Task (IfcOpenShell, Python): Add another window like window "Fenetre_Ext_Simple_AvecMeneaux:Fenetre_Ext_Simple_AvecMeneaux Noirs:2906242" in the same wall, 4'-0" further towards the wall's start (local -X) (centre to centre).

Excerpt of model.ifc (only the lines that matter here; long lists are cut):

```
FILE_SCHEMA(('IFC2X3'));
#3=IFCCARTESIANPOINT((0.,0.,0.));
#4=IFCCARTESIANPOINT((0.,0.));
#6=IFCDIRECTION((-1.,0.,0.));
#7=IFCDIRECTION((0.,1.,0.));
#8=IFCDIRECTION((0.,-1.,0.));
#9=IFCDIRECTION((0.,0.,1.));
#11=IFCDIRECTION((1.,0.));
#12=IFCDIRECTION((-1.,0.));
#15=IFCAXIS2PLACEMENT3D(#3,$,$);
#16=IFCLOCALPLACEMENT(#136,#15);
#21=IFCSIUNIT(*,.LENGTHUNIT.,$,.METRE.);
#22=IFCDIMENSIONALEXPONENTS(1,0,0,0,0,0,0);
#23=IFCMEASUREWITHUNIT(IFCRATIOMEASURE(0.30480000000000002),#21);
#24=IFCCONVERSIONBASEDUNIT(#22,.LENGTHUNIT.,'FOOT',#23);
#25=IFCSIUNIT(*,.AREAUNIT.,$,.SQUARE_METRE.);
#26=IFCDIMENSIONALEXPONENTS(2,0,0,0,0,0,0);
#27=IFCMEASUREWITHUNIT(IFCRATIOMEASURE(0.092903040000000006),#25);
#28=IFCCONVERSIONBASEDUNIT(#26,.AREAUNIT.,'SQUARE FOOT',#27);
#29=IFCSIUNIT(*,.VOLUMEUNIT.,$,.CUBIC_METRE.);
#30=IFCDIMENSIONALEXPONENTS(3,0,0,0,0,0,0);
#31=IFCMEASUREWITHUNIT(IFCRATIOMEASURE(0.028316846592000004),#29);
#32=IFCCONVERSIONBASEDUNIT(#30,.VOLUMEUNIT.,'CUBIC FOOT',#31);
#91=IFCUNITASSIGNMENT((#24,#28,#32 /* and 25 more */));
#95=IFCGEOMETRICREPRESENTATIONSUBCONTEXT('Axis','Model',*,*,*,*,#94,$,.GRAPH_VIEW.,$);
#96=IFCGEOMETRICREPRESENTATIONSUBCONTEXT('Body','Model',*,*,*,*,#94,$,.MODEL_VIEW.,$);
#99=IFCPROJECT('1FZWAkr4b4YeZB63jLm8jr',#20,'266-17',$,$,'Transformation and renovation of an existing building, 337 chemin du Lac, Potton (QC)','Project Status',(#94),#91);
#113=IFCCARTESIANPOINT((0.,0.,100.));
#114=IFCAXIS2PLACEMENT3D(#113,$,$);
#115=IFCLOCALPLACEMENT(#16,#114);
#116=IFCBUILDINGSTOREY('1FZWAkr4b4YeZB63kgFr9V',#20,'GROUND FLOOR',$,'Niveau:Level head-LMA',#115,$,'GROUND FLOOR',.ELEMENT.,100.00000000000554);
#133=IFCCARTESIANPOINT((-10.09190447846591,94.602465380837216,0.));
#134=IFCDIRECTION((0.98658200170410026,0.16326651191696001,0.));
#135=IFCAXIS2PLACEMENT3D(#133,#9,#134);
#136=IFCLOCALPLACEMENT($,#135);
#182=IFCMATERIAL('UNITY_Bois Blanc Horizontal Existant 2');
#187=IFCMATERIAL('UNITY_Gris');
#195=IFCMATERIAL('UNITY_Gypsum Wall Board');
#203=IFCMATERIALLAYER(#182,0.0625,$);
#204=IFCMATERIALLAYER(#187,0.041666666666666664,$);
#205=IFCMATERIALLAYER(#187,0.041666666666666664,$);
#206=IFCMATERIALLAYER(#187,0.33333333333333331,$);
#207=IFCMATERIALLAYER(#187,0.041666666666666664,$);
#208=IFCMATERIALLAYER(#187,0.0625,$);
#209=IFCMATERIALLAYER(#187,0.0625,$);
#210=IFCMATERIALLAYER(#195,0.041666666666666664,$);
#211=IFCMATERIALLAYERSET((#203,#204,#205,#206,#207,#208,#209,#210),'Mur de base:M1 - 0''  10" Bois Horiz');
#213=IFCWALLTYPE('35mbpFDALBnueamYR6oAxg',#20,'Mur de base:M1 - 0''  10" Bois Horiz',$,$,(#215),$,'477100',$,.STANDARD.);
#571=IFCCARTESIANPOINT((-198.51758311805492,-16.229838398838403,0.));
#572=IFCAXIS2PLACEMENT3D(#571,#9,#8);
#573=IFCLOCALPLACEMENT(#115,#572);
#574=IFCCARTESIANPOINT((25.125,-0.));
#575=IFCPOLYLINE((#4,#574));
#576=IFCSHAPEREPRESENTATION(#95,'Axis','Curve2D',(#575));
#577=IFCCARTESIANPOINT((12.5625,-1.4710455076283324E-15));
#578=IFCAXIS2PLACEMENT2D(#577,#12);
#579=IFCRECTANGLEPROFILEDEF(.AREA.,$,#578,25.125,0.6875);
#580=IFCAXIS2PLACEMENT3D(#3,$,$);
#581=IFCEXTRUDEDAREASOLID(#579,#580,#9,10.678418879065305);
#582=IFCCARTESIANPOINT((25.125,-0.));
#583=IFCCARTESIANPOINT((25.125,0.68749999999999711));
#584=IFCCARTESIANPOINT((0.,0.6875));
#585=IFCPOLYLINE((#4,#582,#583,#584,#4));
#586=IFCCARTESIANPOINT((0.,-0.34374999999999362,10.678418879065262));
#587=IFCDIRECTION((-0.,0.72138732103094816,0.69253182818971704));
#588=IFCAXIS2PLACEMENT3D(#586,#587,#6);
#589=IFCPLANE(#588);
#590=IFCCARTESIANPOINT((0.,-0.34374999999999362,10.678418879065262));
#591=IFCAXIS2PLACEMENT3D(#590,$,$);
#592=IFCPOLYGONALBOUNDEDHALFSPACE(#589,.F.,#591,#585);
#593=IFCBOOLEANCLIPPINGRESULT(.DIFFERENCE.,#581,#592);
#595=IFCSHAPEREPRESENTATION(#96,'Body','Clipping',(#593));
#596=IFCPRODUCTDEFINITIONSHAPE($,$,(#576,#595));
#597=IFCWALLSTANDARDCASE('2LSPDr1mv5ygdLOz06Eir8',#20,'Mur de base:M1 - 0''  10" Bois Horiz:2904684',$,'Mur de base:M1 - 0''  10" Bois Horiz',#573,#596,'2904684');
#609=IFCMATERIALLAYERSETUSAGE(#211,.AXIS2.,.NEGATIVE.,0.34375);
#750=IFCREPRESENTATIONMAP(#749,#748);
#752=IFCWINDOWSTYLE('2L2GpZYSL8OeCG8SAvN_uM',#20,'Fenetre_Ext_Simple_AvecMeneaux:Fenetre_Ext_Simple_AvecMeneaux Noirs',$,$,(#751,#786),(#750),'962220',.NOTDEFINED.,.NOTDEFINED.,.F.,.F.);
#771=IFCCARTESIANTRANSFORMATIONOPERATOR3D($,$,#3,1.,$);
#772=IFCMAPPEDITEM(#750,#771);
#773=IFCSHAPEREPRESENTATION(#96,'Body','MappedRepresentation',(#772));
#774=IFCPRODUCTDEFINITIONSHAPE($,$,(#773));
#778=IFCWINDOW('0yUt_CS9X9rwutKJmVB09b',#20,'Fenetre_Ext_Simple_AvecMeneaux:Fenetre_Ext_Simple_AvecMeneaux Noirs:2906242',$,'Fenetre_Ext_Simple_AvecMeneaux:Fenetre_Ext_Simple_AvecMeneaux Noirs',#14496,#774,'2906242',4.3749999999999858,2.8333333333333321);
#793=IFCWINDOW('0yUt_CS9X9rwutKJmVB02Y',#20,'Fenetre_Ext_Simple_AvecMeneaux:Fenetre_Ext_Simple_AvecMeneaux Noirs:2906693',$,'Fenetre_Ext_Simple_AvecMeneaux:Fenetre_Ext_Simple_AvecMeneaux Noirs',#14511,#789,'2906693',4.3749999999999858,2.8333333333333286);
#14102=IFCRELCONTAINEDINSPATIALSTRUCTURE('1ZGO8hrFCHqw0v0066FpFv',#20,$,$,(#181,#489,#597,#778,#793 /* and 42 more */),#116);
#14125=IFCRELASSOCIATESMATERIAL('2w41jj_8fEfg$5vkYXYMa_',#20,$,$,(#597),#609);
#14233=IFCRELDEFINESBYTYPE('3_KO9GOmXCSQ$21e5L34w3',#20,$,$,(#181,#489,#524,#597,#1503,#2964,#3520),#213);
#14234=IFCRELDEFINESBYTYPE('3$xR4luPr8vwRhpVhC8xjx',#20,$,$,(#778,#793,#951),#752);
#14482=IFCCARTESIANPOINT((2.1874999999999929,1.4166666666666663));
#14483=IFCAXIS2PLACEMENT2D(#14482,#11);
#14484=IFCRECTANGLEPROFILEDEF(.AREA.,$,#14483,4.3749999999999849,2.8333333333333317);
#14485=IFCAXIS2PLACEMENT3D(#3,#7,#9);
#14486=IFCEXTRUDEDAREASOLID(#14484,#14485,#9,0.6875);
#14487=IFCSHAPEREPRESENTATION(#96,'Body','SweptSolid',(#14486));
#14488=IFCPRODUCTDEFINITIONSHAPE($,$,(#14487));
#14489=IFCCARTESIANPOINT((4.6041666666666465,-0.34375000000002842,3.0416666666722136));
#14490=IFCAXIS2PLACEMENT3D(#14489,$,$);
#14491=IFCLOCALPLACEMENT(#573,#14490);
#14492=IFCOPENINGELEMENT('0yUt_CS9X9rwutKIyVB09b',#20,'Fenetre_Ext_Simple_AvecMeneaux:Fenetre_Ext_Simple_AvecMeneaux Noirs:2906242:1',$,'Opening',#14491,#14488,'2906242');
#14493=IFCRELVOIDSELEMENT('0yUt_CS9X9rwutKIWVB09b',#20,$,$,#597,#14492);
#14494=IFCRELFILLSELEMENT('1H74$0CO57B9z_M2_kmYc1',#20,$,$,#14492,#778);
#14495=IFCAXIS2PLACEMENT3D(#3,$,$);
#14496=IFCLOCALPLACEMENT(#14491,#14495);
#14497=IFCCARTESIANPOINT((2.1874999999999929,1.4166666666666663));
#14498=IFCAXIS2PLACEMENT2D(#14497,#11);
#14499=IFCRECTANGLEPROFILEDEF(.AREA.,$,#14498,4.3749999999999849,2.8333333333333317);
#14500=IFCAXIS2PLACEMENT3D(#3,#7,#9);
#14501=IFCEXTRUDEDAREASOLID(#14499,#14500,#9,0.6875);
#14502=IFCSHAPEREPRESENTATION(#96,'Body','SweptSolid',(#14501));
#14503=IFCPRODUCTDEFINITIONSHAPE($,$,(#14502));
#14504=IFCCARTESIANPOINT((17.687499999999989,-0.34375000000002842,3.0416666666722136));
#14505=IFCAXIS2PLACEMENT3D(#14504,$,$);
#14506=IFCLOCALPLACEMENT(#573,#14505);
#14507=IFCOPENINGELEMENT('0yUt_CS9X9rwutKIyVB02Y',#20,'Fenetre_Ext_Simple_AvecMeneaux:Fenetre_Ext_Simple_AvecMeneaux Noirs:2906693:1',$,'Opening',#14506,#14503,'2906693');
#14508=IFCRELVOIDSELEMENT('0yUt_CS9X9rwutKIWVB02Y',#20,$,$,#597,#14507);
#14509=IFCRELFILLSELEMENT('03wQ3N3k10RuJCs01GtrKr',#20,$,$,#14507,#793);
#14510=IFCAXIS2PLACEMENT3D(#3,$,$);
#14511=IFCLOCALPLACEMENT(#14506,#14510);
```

```python
import ifcopenshell
import ifcopenshell.api.feature
import ifcopenshell.api.geometry
import ifcopenshell.api.root
import ifcopenshell.geom
import ifcopenshell.util.element
import ifcopenshell.util.placement
import ifcopenshell.util.shape
import ifcopenshell.util.unit

model = ifcopenshell.open("model.ifc")
unit_scale = ifcopenshell.util.unit.calculate_unit_scale(model)
settings = ifcopenshell.geom.settings()


def volume(element):
    """Net volume in cubic metres, openings subtracted."""
    shape = ifcopenshell.geom.create_shape(settings, element)
    return ifcopenshell.util.shape.get_volume(shape.geometry)


def reuse_history(source, copy):
    """copy_class also copies each property set's owner history, people and application; keep the originals."""
    for rel in copy.IsDefinedBy:
        if rel.is_a("IfcRelDefinesByProperties") and (history := rel.RelatingPropertyDefinition.OwnerHistory):
            rel.RelatingPropertyDefinition.OwnerHistory = source.OwnerHistory
            ifcopenshell.util.element.remove_deep2(model, history)


window = model.by_id(778)
opening = window.FillsVoids[0].RelatingOpeningElement
wall = opening.VoidsElements[0].RelatingBuildingElement
before = volume(wall)
shift = ifcopenshell.util.placement.get_local_placement(wall.ObjectPlacement)[:3, 0] * -48 * 0.0254 / unit_scale

# copy_class copies the void relationship, type, container and properties, but no geometry.
new_opening = ifcopenshell.api.root.copy_class(model, product=opening)
new_opening.Representation = ifcopenshell.util.element.copy_deep(
    model, opening.Representation, exclude=["IfcGeometricRepresentationContext", "IfcRepresentationMap"]
)
new_opening.Name = "Fenetre_Ext_Simple_AvecMeneaux:Fenetre_Ext_Simple_AvecMeneaux Noirs"
new_opening.Tag = None
new_window = ifcopenshell.api.root.copy_class(model, product=window)
new_window.Representation = ifcopenshell.util.element.copy_deep(
    model, window.Representation, exclude=["IfcGeometricRepresentationContext", "IfcRepresentationMap"]
)
new_window.Name = "Fenetre_Ext_Simple_AvecMeneaux:Fenetre_Ext_Simple_AvecMeneaux Noirs"
new_window.Tag = None
reuse_history(window, new_window)
fills = ifcopenshell.api.feature.add_filling(model, opening=new_opening, element=new_window)
fills.OwnerHistory = new_window.OwnerHistory  # required in IFC2X3

for old, new in ((opening, new_opening), (window, new_window)):
    matrix = ifcopenshell.util.placement.get_local_placement(old.ObjectPlacement)
    matrix[:3, 3] += shift
    ifcopenshell.api.geometry.edit_object_placement(model, product=new, matrix=matrix, is_si=False)

after = volume(wall)

print(f"wall volume {before:.3f} -> {after:.3f} m3")

model.write("model-out.ifc")
```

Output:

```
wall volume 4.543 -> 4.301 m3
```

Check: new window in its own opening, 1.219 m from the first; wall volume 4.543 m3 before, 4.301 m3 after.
